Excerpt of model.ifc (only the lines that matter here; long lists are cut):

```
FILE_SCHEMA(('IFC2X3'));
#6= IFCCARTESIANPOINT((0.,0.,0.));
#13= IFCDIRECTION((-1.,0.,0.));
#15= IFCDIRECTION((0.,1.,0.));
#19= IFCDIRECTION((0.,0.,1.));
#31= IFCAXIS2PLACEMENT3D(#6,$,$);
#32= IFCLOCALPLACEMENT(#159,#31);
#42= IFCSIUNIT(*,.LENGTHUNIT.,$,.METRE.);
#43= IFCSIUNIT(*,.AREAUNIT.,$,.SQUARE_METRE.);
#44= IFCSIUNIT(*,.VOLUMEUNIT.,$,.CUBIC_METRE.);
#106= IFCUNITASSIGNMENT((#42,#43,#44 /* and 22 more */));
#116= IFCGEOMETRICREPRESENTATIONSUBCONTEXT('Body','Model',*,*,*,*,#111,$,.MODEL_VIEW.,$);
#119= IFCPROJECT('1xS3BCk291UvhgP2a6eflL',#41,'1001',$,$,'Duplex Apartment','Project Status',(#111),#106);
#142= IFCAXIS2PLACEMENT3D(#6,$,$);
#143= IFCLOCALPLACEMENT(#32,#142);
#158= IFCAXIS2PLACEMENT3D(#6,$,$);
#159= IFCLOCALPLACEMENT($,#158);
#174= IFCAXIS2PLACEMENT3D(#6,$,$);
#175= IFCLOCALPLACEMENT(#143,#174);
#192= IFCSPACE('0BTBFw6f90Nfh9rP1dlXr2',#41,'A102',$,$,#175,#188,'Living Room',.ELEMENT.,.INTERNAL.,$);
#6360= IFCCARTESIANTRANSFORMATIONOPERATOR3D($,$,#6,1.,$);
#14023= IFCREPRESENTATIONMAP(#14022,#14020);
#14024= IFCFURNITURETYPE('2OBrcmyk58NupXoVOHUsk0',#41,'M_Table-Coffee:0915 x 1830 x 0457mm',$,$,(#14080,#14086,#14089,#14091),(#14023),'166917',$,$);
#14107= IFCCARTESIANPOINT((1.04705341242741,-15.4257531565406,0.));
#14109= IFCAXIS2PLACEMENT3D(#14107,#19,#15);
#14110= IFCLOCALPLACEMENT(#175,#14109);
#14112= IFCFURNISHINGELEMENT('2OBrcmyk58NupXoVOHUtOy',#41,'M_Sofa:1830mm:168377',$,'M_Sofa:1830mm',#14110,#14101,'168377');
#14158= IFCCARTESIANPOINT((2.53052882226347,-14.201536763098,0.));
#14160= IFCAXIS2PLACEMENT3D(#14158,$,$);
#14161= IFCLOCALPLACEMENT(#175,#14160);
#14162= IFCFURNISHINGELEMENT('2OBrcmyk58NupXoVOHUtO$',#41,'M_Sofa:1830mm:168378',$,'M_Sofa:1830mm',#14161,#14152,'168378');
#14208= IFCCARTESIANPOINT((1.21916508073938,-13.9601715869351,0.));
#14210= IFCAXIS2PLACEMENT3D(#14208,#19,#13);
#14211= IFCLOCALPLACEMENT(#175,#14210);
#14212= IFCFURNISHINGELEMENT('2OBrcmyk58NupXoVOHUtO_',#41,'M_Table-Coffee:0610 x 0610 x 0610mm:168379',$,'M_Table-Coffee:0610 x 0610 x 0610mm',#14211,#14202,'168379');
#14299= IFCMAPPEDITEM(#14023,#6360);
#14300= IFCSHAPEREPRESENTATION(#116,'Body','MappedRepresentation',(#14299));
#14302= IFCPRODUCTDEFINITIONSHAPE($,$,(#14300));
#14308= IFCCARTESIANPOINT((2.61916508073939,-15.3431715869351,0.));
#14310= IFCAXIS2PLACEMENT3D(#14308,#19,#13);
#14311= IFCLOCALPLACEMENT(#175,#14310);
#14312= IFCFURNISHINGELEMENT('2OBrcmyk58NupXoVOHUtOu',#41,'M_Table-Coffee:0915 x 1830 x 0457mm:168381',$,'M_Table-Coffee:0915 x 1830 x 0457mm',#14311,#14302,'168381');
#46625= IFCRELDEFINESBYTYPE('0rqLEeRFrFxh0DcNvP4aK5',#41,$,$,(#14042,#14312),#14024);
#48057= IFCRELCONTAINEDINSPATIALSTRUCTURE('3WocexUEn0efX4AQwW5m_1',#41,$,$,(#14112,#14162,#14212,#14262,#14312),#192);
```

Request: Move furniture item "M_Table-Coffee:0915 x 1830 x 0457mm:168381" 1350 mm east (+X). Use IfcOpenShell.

```python
import ifcopenshell
import ifcopenshell.api.geometry
import ifcopenshell.util.placement
import ifcopenshell.util.unit

model = ifcopenshell.open("model.ifc")
unit_scale = ifcopenshell.util.unit.calculate_unit_scale(model)

item = model.by_id(14312)
matrix = ifcopenshell.util.placement.get_local_placement(item.ObjectPlacement)
matrix[0, 3] += 1.35 / unit_scale
ifcopenshell.api.geometry.edit_object_placement(model, product=item, matrix=matrix, is_si=False)

print(ifcopenshell.util.placement.get_local_placement(item.ObjectPlacement).round(3) + 0.0)

model.write("model_updated.ifc")
```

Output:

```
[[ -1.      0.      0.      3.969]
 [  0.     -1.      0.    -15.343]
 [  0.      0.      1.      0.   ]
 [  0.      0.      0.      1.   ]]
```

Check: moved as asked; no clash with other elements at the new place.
